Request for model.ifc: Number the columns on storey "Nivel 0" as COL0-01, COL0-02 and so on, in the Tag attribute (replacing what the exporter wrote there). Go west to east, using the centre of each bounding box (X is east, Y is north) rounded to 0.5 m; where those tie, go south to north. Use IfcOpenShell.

First a look at what the model holds.

```python
import ifcopenshell
import ifcopenshell.util.element
import ifcopenshell.util.placement

model = ifcopenshell.open("model.ifc")
print(model.schema)
storey = next(s for s in model.by_type("IfcBuildingStorey") if s.Name == "Nivel 0")
columns = [e for e in ifcopenshell.util.element.get_decomposition(storey) if e.is_a("IfcColumn")]
for e in sorted(columns, key=lambda e: e.id()):
    origin = ifcopenshell.util.placement.get_local_placement(e.ObjectPlacement)[:3, 3]
    print(e.id(), e.Tag, e.Name, origin.round(2) + 0.0, sep=" | ")
```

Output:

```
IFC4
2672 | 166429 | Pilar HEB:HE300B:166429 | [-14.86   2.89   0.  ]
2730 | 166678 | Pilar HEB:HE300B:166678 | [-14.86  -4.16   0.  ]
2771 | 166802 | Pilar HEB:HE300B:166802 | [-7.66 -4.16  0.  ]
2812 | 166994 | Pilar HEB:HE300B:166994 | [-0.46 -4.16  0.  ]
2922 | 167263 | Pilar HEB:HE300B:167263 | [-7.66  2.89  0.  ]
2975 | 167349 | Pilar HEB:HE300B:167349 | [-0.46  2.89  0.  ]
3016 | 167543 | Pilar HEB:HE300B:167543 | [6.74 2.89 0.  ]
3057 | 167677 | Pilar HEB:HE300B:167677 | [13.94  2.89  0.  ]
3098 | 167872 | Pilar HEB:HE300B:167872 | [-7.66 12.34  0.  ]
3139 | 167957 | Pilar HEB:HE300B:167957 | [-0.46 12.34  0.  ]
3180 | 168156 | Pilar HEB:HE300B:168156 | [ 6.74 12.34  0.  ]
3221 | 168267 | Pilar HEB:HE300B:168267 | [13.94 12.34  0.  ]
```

```python
import ifcopenshell
import ifcopenshell.geom
import ifcopenshell.util.element
import ifcopenshell.util.shape

model = ifcopenshell.open("model.ifc")
settings = ifcopenshell.geom.settings()
settings.set("use-world-coords", True)


def centre(element):
    shape = ifcopenshell.geom.create_shape(settings, element)
    return ifcopenshell.util.shape.get_bbox_centroid(shape.geometry)


storey = next(s for s in model.by_type("IfcBuildingStorey") if s.Name == "Nivel 0")
columns = [e for e in ifcopenshell.util.element.get_decomposition(storey) if e.is_a("IfcColumn")]

# Insertion points can sit at a corner or the storey origin, so sort by the geometry (in metres).
centres = {e: centre(e) for e in columns}
columns.sort(key=lambda e: (round(centres[e][0] / 0.5), centres[e][1]))

for i, e in enumerate(columns, start=1):
    number = f"COL0-{i:02d}"
    e.Tag = number
    print(e.id(), number)

model.write("model_v2.ifc")
```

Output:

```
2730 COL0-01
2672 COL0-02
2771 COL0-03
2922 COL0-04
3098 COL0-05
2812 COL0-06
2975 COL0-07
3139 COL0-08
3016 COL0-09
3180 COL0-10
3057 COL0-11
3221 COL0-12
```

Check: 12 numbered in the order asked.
